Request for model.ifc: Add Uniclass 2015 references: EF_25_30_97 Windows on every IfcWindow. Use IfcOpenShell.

First a look at what the model holds.

```python
import ifcopenshell

model = ifcopenshell.open("model.ifc")
print(model.schema)
print("classifications:", [c.Name for c in model.by_type("IfcClassification")])
for ifc_class in ("IfcDoor", "IfcRoof", "IfcStair", "IfcWall", "IfcWindow"):
    print(ifc_class, len(model.by_type(ifc_class)))
```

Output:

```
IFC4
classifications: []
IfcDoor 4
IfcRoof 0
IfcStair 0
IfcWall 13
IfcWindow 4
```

```python
import ifcopenshell
import ifcopenshell.api.classification

model = ifcopenshell.open("model.ifc")

system = ifcopenshell.api.classification.add_classification(model, classification="Uniclass 2015")

codes = {
    "IfcWindow": ("EF_25_30_97", "Windows"),
}
for ifc_class, (code, name) in codes.items():
    products = model.by_type(ifc_class)
    ifcopenshell.api.classification.add_reference(
        model, products=products, classification=system, identification=code, name=name
    )
    print(code, len(products))

model.write("model_edited.ifc")
```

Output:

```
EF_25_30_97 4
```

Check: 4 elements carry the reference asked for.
